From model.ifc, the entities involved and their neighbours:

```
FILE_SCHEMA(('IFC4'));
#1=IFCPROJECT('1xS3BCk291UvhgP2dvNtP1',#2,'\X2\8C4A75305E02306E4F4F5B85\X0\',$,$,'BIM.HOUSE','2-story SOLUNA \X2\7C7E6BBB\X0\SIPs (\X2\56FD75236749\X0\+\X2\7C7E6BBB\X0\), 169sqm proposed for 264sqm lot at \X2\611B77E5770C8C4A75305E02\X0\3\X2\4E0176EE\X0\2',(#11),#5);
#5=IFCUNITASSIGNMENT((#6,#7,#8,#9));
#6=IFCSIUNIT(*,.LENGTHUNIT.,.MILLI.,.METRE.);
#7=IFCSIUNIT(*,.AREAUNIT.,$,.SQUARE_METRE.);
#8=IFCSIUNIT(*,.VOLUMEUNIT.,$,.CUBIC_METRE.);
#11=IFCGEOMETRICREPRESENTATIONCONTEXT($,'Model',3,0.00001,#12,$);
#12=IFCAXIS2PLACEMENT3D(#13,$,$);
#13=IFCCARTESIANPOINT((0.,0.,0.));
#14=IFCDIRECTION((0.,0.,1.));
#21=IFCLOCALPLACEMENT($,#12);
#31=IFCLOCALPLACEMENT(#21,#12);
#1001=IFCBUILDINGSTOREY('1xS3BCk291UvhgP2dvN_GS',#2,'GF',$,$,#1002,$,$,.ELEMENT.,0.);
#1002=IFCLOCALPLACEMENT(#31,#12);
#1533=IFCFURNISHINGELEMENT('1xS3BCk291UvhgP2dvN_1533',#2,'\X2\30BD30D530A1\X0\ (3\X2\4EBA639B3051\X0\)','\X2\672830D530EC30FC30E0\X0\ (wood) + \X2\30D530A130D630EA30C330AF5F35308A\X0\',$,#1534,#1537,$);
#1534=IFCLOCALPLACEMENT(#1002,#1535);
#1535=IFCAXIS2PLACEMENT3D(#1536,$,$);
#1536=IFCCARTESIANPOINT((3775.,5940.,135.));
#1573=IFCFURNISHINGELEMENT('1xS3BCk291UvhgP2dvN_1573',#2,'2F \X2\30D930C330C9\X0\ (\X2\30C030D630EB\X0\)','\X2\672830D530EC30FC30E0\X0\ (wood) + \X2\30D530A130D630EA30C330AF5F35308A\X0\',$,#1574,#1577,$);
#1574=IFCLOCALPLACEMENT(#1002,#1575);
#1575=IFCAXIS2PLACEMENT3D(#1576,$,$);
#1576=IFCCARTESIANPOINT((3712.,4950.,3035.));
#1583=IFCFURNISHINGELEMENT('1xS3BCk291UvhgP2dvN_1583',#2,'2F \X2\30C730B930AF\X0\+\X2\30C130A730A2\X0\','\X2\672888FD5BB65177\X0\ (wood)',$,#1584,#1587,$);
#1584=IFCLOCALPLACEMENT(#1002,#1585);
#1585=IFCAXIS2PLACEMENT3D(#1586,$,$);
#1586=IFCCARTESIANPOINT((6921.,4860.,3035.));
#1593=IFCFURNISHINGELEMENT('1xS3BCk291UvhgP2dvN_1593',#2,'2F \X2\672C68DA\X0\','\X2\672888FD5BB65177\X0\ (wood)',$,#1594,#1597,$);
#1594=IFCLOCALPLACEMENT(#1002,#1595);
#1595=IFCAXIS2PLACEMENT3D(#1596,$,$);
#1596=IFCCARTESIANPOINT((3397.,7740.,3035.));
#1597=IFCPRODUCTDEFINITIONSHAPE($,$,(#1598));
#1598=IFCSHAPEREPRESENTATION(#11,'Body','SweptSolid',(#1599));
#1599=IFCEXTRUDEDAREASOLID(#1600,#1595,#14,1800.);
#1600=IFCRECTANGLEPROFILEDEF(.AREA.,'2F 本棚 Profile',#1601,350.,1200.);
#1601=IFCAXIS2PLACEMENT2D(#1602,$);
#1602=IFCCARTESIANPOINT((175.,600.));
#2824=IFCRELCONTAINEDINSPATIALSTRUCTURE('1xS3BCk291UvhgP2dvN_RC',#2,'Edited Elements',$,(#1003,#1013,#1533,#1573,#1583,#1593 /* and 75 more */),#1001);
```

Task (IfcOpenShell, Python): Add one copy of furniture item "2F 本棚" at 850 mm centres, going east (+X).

```python
import numpy as np
import ifcopenshell
import ifcopenshell.api.geometry
import ifcopenshell.api.root
import ifcopenshell.util.element
import ifcopenshell.util.placement

model = ifcopenshell.open("model.ifc")


def reuse_history(source, copy):
    """copy_class also copies each property set's owner history, people and application; keep the originals."""
    for rel in copy.IsDefinedBy:
        if rel.is_a("IfcRelDefinesByProperties") and (history := rel.RelatingPropertyDefinition.OwnerHistory):
            rel.RelatingPropertyDefinition.OwnerHistory = source.OwnerHistory
            ifcopenshell.util.element.remove_deep2(model, history)


source = model.by_guid("1xS3BCk291UvhgP2dvN_1593")
base = ifcopenshell.util.placement.get_local_placement(source.ObjectPlacement)
step = np.array([1.0, 0.0, 0.0]) * 850.0

for i in range(1, 2):
    copy = ifcopenshell.api.root.copy_class(model, product=source)
    copy.Representation = ifcopenshell.util.element.copy_deep(
        model, source.Representation, exclude=["IfcGeometricRepresentationContext", "IfcRepresentationMap"]
    )
    reuse_history(source, copy)
    matrix = base.copy()
    matrix[:3, 3] += i * step
    print("added at", matrix[:3, 3].round(3) + 0.0)
    ifcopenshell.api.geometry.edit_object_placement(model, product=copy, matrix=matrix, is_si=False)

model.write("model_rev.ifc")
```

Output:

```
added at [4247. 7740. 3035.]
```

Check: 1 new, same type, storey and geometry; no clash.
